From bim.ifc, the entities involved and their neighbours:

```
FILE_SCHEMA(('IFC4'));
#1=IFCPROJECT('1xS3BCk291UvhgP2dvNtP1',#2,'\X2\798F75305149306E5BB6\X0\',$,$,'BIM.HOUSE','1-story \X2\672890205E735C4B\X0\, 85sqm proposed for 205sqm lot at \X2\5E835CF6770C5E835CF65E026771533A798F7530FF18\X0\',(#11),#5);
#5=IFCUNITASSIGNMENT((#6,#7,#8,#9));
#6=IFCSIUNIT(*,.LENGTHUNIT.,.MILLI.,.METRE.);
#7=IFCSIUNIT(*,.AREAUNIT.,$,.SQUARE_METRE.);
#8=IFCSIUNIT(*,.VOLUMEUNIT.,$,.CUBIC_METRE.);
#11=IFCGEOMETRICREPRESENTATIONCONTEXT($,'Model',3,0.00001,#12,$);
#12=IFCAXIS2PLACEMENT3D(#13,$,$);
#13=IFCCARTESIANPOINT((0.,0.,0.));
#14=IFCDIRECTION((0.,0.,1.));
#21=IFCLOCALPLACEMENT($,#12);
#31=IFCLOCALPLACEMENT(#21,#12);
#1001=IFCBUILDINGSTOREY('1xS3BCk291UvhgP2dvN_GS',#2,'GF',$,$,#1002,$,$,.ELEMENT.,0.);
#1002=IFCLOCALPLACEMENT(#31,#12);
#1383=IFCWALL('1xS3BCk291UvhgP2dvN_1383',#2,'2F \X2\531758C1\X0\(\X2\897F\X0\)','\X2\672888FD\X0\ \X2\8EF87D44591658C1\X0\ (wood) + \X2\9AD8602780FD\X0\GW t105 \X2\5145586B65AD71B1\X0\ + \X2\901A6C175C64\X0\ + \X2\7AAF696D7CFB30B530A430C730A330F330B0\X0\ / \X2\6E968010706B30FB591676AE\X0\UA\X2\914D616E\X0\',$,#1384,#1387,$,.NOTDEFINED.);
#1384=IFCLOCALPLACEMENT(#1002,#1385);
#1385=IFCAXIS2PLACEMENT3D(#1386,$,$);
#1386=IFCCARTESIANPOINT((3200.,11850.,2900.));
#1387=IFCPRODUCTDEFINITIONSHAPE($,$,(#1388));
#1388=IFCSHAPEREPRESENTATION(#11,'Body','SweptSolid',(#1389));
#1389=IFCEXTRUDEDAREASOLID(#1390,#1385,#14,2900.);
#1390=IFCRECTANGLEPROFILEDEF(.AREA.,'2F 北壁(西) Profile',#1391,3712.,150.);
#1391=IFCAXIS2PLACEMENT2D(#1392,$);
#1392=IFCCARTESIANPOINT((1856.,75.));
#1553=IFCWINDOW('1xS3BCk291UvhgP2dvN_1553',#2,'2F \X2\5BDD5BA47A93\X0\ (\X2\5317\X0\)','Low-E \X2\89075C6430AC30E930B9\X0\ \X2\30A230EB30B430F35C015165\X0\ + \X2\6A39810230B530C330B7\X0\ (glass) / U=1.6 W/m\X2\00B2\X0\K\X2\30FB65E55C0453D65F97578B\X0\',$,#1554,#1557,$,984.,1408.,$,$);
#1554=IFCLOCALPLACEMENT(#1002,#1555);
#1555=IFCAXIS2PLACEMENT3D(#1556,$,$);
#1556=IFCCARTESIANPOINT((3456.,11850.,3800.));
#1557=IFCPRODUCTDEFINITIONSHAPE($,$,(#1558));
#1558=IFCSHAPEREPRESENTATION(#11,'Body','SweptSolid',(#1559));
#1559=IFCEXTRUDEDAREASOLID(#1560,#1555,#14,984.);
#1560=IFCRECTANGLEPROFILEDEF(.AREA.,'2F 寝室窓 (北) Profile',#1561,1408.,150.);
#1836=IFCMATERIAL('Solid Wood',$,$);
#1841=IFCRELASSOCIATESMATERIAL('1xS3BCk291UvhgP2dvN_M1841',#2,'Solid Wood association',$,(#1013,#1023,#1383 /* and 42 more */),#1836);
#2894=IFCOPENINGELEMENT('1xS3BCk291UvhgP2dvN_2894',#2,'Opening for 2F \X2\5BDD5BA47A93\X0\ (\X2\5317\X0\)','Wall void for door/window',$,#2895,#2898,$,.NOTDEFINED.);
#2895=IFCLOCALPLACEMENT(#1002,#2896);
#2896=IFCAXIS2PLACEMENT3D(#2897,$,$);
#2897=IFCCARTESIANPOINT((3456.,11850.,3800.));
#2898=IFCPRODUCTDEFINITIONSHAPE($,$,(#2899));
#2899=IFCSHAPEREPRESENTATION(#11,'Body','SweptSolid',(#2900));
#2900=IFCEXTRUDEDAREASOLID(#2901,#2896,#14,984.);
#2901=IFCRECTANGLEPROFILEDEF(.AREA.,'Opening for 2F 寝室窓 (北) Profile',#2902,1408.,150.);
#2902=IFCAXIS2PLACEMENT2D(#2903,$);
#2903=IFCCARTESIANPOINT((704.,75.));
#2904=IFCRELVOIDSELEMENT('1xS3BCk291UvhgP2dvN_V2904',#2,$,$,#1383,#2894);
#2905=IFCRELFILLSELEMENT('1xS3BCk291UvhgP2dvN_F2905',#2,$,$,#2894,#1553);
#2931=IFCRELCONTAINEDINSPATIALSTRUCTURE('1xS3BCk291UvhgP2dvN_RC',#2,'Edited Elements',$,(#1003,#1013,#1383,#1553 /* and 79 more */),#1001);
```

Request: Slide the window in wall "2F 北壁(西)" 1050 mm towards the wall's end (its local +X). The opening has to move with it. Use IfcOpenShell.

```python
import ifcopenshell
import ifcopenshell.api.geometry
import ifcopenshell.util.placement

model = ifcopenshell.open("bim.ifc")

window = model.by_id(1553)
opening = window.FillsVoids[0].RelatingOpeningElement
wall = opening.VoidsElements[0].RelatingBuildingElement

wall_matrix = ifcopenshell.util.placement.get_local_placement(wall.ObjectPlacement)
shift = wall_matrix[:3, 0] * 1050.0
before = ifcopenshell.util.placement.get_local_placement(window.ObjectPlacement)[:3, 3].copy()

# The window is not placed relative to its opening, so move both.
for product in (opening, window):
    matrix = ifcopenshell.util.placement.get_local_placement(product.ObjectPlacement)
    matrix[:3, 3] += shift
    ifcopenshell.api.geometry.edit_object_placement(model, product=product, matrix=matrix, is_si=False)

after = ifcopenshell.util.placement.get_local_placement(window.ObjectPlacement)[:3, 3]
print("window moved by", (after - before).round(3) + 0.0)

model.write("bim_v2.ifc")
```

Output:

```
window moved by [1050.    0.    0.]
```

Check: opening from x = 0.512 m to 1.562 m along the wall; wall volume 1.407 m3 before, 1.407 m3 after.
